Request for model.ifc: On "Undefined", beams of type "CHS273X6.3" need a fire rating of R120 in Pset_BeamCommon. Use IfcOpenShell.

First a look at what the model holds.

```python
import ifcopenshell
import ifcopenshell.util.element

model = ifcopenshell.open("model.ifc")
print(model.schema)
storey = next(s for s in model.by_type("IfcBuildingStorey") if s.Name == "Undefined")
beams = [e for e in ifcopenshell.util.element.get_decomposition(storey) if e.is_a("IfcBeam")]
seen = {}
for e in beams:
    element_type = ifcopenshell.util.element.get_type(e)
    key = (element_type.Name if element_type != e and element_type else None, ifcopenshell.util.element.get_pset(e, "Pset_BeamCommon", "FireRating"))
    seen[key] = seen.get(key, 0) + 1
for (name, value), count in sorted(seen.items(), key=str):
    print(count, "x", name, "|", value)
```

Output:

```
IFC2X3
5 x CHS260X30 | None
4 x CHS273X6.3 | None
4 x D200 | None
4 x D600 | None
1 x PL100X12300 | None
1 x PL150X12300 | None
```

```python
import ifcopenshell
import ifcopenshell.api.pset
import ifcopenshell.util.element

model = ifcopenshell.open("model.ifc")

storey = next(s for s in model.by_type("IfcBuildingStorey") if s.Name == "Undefined")
beams = [e for e in ifcopenshell.util.element.get_decomposition(storey) if e.is_a("IfcBeam")]

count = 0
for e in beams:
    element_type = ifcopenshell.util.element.get_type(e)
    if element_type in (None, e) or element_type.Name != "CHS273X6.3":
        continue
    found = ifcopenshell.util.element.get_pset(e, "Pset_BeamCommon", should_inherit=False)
    if found:
        pset = model.by_id(found["id"])
        if len(ifcopenshell.util.element.get_elements_by_pset(pset)) > 1:
            pset = ifcopenshell.api.pset.unshare_pset(model, products=[e], pset=pset)[0]
    else:
        pset = ifcopenshell.api.pset.add_pset(model, product=e, name="Pset_BeamCommon")
    ifcopenshell.api.pset.edit_pset(model, pset=pset, properties={"FireRating": "R120"})
    count += 1

print(count, "beams updated")

model.write("model_updated.ifc")
```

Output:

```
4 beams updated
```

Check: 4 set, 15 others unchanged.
